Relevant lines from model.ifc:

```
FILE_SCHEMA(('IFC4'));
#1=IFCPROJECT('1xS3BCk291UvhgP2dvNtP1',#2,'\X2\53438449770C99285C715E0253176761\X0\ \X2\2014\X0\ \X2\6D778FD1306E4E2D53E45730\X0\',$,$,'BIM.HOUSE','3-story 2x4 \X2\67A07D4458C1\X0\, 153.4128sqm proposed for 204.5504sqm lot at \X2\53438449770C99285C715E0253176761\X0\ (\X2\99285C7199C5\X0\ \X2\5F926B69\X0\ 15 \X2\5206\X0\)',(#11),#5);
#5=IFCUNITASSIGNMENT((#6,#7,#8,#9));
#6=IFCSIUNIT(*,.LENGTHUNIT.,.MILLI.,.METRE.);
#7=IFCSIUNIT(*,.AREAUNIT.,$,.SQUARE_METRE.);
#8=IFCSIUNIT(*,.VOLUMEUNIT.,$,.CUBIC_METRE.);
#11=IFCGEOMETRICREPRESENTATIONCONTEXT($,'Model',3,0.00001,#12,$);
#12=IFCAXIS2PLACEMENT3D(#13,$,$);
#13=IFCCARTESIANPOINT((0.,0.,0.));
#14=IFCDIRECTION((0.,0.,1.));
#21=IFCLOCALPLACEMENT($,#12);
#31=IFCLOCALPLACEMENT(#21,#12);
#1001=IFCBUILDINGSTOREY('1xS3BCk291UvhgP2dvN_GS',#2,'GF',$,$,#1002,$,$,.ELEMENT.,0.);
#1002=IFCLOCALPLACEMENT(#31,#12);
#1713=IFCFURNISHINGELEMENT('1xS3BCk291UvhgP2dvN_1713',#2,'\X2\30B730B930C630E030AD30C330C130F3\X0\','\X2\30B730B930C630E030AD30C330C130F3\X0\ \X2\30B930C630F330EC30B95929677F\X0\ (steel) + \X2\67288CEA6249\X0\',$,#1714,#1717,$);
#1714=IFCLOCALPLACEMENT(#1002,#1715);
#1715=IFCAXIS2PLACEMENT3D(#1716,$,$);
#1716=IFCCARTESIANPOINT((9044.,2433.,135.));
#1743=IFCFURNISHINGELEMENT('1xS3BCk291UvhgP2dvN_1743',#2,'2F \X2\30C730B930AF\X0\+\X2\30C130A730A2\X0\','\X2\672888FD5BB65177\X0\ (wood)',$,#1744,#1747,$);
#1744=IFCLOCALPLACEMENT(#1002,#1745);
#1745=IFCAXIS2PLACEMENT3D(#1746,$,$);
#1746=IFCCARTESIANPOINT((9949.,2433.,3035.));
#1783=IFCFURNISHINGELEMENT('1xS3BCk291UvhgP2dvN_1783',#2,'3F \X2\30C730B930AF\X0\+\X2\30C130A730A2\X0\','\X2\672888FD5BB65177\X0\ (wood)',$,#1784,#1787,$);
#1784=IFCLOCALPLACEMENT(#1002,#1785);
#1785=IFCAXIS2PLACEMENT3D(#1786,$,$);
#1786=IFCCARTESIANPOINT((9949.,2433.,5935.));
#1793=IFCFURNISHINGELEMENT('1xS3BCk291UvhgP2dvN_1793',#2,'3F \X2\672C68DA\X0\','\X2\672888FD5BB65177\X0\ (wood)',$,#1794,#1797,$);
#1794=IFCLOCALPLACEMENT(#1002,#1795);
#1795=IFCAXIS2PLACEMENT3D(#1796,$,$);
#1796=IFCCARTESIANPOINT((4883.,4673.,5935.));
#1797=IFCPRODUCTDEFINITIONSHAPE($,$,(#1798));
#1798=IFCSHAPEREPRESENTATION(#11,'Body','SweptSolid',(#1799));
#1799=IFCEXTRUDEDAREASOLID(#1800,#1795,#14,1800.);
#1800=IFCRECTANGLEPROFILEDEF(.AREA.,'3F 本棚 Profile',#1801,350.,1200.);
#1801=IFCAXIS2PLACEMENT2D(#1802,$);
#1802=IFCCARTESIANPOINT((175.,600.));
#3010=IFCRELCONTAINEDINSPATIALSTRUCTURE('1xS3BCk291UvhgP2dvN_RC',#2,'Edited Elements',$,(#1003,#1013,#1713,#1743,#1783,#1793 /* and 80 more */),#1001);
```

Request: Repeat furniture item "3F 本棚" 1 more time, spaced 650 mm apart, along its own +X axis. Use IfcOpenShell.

```python
import ifcopenshell
import ifcopenshell.api.geometry
import ifcopenshell.api.root
import ifcopenshell.util.element
import ifcopenshell.util.placement
import ifcopenshell.util.unit

model = ifcopenshell.open("model.ifc")
unit_scale = ifcopenshell.util.unit.calculate_unit_scale(model)


def reuse_history(source, copy):
    """copy_class also copies each property set's owner history, people and application; keep the originals."""
    for rel in copy.IsDefinedBy:
        if rel.is_a("IfcRelDefinesByProperties") and (history := rel.RelatingPropertyDefinition.OwnerHistory):
            rel.RelatingPropertyDefinition.OwnerHistory = source.OwnerHistory
            ifcopenshell.util.element.remove_deep2(model, history)


source = model.by_id(1793)
base = ifcopenshell.util.placement.get_local_placement(source.ObjectPlacement)
step = base[:3, 0] * 0.65 / unit_scale

for i in range(1, 2):
    copy = ifcopenshell.api.root.copy_class(model, product=source)
    copy.Representation = ifcopenshell.util.element.copy_deep(
        model, source.Representation, exclude=["IfcGeometricRepresentationContext", "IfcRepresentationMap"]
    )
    reuse_history(source, copy)
    matrix = base.copy()
    matrix[:3, 3] += i * step
    print("added at", matrix[:3, 3].round(3) + 0.0)
    ifcopenshell.api.geometry.edit_object_placement(model, product=copy, matrix=matrix, is_si=False)

model.write("model_v2.ifc")
```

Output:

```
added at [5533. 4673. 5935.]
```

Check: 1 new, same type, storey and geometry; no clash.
